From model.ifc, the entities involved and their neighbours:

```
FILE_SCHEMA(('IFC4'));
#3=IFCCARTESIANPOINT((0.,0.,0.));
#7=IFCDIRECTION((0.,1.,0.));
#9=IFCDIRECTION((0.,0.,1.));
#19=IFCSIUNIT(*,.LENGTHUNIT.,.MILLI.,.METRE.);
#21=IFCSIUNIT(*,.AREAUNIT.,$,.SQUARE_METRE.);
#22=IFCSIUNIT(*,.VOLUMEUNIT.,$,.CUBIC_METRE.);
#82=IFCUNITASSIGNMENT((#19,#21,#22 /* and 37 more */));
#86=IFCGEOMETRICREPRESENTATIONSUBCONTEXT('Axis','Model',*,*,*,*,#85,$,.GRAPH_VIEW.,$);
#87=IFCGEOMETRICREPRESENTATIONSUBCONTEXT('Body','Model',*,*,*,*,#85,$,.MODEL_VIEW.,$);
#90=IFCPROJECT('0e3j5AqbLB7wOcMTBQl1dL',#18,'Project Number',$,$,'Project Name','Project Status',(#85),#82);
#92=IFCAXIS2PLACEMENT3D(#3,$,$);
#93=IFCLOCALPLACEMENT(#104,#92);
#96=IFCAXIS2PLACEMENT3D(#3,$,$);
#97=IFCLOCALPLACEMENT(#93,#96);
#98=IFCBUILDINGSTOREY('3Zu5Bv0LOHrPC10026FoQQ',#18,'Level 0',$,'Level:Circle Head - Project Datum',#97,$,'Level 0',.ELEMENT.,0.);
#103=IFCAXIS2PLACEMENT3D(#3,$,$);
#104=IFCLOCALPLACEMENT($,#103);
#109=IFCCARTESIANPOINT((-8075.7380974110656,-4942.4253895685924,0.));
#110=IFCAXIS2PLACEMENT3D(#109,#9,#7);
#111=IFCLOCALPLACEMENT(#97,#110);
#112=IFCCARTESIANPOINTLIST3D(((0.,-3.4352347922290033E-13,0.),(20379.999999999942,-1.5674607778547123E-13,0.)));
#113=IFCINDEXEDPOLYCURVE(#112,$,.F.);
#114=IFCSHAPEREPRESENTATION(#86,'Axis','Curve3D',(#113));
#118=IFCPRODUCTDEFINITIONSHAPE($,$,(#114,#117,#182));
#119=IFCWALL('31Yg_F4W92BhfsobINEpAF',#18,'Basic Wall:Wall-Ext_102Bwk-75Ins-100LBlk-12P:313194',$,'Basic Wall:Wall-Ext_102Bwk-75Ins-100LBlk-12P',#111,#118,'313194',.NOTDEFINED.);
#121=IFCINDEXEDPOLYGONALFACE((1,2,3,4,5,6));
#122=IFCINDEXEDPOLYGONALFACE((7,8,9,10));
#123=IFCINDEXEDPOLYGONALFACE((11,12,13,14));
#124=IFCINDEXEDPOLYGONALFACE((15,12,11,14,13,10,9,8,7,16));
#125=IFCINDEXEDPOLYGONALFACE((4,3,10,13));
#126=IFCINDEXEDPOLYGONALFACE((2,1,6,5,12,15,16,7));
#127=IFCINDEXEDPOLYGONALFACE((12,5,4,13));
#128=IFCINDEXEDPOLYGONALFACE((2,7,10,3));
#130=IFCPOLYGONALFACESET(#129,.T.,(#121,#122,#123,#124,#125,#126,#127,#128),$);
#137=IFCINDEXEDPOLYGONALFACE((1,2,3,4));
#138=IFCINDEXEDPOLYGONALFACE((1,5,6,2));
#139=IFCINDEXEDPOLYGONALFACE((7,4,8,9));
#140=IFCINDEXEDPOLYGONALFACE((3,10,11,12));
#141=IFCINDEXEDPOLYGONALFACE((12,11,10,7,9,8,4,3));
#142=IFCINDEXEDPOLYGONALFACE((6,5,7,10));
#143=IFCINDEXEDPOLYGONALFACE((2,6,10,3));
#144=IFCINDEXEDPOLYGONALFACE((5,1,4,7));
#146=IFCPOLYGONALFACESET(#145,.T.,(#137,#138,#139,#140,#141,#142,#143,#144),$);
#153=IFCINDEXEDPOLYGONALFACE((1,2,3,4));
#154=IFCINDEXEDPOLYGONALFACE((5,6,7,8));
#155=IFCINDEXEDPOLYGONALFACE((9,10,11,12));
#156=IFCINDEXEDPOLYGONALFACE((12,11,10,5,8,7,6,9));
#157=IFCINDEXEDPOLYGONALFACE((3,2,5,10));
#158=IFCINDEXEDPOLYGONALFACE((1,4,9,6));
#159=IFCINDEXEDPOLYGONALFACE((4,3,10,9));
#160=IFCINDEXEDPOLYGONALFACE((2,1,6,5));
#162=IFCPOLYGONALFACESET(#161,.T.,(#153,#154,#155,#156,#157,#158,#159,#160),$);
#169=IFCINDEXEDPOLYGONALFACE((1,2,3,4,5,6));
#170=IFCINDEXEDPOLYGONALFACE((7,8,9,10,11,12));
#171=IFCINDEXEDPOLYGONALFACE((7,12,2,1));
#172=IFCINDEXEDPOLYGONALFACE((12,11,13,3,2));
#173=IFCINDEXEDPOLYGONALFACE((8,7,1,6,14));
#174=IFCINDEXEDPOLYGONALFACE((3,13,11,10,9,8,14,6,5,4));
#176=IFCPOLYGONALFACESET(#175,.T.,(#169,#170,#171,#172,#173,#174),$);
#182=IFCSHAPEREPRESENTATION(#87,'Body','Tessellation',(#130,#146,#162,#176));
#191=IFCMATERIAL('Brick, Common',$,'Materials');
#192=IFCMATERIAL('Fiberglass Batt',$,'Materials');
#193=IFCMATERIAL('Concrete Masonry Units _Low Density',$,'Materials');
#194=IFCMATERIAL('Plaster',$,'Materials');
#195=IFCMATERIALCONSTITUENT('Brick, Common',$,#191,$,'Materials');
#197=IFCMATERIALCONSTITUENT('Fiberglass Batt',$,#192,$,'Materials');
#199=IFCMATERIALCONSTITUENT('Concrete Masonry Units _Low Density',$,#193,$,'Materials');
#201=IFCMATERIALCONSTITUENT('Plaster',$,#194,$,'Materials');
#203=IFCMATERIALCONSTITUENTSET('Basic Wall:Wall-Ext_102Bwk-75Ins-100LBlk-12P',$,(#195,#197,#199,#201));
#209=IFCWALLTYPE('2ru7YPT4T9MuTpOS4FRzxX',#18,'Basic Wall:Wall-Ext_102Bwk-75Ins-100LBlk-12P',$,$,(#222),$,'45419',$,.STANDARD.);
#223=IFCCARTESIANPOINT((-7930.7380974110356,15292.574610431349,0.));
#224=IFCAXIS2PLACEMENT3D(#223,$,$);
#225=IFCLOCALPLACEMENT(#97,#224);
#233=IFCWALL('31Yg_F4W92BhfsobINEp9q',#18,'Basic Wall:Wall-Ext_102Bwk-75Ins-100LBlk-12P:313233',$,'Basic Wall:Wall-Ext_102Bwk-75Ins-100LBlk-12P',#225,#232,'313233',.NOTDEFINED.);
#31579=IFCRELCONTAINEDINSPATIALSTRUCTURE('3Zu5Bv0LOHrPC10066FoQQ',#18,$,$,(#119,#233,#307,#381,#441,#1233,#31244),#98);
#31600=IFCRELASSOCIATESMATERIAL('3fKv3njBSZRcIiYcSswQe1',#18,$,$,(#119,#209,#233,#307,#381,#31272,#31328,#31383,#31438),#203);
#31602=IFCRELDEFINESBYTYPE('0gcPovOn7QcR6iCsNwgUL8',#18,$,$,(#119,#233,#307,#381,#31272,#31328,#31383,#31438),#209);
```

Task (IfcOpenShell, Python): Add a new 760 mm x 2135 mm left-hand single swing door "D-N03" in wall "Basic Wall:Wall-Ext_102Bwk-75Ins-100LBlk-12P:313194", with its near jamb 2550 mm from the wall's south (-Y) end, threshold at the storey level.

```python
import numpy as np
import ifcopenshell
import ifcopenshell.api.feature
import ifcopenshell.api.geometry
import ifcopenshell.api.root
import ifcopenshell.api.spatial
import ifcopenshell.geom
import ifcopenshell.util.element
import ifcopenshell.util.placement
import ifcopenshell.util.representation
import ifcopenshell.util.shape
import ifcopenshell.util.unit

model = ifcopenshell.open("model.ifc")
unit_scale = ifcopenshell.util.unit.calculate_unit_scale(model)
settings = ifcopenshell.geom.settings()


def volume(element):
    """Net volume in cubic metres, openings subtracted."""
    shape = ifcopenshell.geom.create_shape(settings, element)
    return ifcopenshell.util.shape.get_volume(shape.geometry)


wall = model.by_id(119)
storey = ifcopenshell.util.element.get_container(wall, ifc_class="IfcBuildingStorey")
context = ifcopenshell.util.representation.get_context(model, "Model", "Body", "MODEL_VIEW")
before = volume(wall)

width, height, from_end, sill = 0.76, 2.135, 2.55, 0.0  # metres

# The wall runs along its own X axis, and the end named is its -X end.
wall_shape = ifcopenshell.geom.create_shape(settings, wall)
x, y, z = ifcopenshell.util.shape.get_vertices(wall_shape.geometry).T
start = x.min() + from_end
face, thickness = float(y.min()), float(y.max() - y.min())
wall_matrix = ifcopenshell.util.placement.get_local_placement(wall.ObjectPlacement)
level = ifcopenshell.util.placement.get_local_placement(storey.ObjectPlacement)[2, 3]


def in_wall(x, y):
    """Placement at x, y metres in the wall's axes, at sill height."""
    matrix = wall_matrix.copy()
    matrix[:, 3] = wall_matrix @ np.array([x / unit_scale, y / unit_scale, 0.0, 1.0])
    matrix[2, 3] = level + sill / unit_scale
    return matrix


# Opening: a box that overshoots both wall faces by 50 mm.
opening = ifcopenshell.api.root.create_entity(model, ifc_class="IfcOpeningElement", predefined_type="OPENING")
box = ifcopenshell.api.geometry.add_wall_representation(
    model, context=context, length=width, height=height, thickness=thickness + 0.1
)
ifcopenshell.api.geometry.assign_representation(model, product=opening, representation=box)
ifcopenshell.api.geometry.edit_object_placement(model, product=opening, matrix=in_wall(start, face - 0.05), is_si=False)
ifcopenshell.api.feature.add_feature(model, feature=opening, element=wall)

door = ifcopenshell.api.root.create_entity(model, ifc_class="IfcDoor", name="D-N03", predefined_type="DOOR")
door.OverallWidth, door.OverallHeight = width / unit_scale, height / unit_scale
door.OperationType = "SINGLE_SWING_LEFT"
body = ifcopenshell.api.geometry.add_door_representation(
    model,
    context=context,
    overall_width=door.OverallWidth,
    overall_height=door.OverallHeight,
    operation_type="SINGLE_SWING_LEFT",
    lining_properties={"LiningDepth": thickness / unit_scale, "ThresholdDepth": thickness / unit_scale},
)
ifcopenshell.api.geometry.assign_representation(model, product=door, representation=body)
ifcopenshell.api.spatial.assign_container(model, products=[door], relating_structure=storey)
ifcopenshell.api.feature.add_filling(model, opening=opening, element=door)

# The lining spans the wall, so the door starts at the wall face.
ifcopenshell.api.geometry.edit_object_placement(model, product=door, matrix=in_wall(start, face), is_si=False)

after = volume(wall)

print(f"wall volume {before:.3f} -> {after:.3f} m3")

model.write("model-out.ifc")
```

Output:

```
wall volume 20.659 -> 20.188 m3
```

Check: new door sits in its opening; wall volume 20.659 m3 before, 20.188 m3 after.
